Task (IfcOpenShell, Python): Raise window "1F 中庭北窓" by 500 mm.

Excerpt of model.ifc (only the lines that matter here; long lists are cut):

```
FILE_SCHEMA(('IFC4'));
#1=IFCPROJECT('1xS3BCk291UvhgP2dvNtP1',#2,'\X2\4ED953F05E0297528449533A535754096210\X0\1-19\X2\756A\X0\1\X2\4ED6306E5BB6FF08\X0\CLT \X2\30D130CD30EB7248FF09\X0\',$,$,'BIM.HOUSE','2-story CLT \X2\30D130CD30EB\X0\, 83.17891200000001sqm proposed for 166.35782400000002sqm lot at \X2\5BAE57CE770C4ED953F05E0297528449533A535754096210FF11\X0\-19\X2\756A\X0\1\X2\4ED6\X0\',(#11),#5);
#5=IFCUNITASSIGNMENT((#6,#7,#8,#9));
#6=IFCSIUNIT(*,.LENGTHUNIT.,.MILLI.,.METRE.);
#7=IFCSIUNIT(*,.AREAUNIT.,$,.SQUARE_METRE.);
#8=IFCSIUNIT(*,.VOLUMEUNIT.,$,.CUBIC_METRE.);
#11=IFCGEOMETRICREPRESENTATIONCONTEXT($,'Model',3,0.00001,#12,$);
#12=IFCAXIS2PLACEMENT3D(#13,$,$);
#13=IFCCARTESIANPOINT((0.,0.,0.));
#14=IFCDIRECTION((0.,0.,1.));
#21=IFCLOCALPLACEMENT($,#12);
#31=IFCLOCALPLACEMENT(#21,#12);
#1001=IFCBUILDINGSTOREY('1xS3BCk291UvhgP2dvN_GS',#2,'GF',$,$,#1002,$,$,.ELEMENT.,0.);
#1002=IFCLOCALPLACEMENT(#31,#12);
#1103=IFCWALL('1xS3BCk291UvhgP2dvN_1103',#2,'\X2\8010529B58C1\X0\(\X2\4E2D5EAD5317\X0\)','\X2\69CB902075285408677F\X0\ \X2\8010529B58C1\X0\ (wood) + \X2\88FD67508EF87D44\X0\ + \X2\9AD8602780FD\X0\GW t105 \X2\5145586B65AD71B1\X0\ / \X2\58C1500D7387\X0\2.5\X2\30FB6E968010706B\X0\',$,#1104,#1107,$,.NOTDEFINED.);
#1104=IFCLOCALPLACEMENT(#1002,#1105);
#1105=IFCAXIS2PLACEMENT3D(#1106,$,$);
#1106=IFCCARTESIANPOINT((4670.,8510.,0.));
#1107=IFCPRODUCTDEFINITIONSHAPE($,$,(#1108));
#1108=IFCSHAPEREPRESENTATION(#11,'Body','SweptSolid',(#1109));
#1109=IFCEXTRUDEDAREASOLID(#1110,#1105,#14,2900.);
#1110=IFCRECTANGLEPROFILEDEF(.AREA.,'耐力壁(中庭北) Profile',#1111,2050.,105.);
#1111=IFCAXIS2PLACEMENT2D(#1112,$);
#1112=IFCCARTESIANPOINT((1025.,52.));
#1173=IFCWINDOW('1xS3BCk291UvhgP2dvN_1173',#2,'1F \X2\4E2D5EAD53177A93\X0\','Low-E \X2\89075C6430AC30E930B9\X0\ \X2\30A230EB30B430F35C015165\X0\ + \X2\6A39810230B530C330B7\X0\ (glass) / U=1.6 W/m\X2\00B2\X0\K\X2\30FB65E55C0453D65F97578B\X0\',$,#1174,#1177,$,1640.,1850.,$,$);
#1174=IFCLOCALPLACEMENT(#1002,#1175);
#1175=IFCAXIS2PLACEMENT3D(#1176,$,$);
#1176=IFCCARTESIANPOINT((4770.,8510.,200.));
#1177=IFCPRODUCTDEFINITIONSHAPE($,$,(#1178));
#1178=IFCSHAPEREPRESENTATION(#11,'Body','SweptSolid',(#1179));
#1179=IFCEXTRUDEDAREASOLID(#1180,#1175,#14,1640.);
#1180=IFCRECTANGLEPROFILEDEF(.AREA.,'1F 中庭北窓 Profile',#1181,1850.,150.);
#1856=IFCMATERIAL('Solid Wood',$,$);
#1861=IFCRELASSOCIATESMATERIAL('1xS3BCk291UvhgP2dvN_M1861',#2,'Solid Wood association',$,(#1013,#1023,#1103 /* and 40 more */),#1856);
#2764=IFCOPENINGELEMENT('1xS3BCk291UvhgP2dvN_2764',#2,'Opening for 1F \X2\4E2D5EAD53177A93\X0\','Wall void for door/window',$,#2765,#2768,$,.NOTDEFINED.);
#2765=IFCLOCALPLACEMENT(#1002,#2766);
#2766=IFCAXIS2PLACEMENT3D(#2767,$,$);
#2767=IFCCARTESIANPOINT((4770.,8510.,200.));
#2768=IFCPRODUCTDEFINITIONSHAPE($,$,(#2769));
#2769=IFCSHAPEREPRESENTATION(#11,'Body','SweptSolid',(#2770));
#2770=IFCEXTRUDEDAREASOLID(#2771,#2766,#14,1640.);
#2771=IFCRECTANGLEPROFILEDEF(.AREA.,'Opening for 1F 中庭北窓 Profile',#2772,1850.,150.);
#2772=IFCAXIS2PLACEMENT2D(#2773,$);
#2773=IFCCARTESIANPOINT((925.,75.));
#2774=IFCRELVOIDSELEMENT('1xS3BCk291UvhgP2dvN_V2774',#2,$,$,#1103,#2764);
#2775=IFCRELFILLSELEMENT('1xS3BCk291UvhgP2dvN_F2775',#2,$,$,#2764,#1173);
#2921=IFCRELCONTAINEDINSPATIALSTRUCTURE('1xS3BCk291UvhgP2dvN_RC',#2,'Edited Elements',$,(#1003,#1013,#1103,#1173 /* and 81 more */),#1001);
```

```python
import numpy as np
import ifcopenshell
import ifcopenshell.api.geometry
import ifcopenshell.util.placement
import ifcopenshell.util.unit

model = ifcopenshell.open("model.ifc")
unit_scale = ifcopenshell.util.unit.calculate_unit_scale(model)

window = model.by_guid("1xS3BCk291UvhgP2dvN_1173")
opening = window.FillsVoids[0].RelatingOpeningElement
dz = 0.5 / unit_scale

shift = np.array([0.0, 0.0, dz])
# The window is not placed relative to its opening, so move both.
for product in (opening, window):
    matrix = ifcopenshell.util.placement.get_local_placement(product.ObjectPlacement)
    matrix[:3, 3] += shift
    ifcopenshell.api.geometry.edit_object_placement(model, product=product, matrix=matrix, is_si=False)

print(f"moved by {dz * unit_scale:+.3f} m")

model.write("model_v2.ifc")
```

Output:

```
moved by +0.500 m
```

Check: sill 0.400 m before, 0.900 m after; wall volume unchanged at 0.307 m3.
